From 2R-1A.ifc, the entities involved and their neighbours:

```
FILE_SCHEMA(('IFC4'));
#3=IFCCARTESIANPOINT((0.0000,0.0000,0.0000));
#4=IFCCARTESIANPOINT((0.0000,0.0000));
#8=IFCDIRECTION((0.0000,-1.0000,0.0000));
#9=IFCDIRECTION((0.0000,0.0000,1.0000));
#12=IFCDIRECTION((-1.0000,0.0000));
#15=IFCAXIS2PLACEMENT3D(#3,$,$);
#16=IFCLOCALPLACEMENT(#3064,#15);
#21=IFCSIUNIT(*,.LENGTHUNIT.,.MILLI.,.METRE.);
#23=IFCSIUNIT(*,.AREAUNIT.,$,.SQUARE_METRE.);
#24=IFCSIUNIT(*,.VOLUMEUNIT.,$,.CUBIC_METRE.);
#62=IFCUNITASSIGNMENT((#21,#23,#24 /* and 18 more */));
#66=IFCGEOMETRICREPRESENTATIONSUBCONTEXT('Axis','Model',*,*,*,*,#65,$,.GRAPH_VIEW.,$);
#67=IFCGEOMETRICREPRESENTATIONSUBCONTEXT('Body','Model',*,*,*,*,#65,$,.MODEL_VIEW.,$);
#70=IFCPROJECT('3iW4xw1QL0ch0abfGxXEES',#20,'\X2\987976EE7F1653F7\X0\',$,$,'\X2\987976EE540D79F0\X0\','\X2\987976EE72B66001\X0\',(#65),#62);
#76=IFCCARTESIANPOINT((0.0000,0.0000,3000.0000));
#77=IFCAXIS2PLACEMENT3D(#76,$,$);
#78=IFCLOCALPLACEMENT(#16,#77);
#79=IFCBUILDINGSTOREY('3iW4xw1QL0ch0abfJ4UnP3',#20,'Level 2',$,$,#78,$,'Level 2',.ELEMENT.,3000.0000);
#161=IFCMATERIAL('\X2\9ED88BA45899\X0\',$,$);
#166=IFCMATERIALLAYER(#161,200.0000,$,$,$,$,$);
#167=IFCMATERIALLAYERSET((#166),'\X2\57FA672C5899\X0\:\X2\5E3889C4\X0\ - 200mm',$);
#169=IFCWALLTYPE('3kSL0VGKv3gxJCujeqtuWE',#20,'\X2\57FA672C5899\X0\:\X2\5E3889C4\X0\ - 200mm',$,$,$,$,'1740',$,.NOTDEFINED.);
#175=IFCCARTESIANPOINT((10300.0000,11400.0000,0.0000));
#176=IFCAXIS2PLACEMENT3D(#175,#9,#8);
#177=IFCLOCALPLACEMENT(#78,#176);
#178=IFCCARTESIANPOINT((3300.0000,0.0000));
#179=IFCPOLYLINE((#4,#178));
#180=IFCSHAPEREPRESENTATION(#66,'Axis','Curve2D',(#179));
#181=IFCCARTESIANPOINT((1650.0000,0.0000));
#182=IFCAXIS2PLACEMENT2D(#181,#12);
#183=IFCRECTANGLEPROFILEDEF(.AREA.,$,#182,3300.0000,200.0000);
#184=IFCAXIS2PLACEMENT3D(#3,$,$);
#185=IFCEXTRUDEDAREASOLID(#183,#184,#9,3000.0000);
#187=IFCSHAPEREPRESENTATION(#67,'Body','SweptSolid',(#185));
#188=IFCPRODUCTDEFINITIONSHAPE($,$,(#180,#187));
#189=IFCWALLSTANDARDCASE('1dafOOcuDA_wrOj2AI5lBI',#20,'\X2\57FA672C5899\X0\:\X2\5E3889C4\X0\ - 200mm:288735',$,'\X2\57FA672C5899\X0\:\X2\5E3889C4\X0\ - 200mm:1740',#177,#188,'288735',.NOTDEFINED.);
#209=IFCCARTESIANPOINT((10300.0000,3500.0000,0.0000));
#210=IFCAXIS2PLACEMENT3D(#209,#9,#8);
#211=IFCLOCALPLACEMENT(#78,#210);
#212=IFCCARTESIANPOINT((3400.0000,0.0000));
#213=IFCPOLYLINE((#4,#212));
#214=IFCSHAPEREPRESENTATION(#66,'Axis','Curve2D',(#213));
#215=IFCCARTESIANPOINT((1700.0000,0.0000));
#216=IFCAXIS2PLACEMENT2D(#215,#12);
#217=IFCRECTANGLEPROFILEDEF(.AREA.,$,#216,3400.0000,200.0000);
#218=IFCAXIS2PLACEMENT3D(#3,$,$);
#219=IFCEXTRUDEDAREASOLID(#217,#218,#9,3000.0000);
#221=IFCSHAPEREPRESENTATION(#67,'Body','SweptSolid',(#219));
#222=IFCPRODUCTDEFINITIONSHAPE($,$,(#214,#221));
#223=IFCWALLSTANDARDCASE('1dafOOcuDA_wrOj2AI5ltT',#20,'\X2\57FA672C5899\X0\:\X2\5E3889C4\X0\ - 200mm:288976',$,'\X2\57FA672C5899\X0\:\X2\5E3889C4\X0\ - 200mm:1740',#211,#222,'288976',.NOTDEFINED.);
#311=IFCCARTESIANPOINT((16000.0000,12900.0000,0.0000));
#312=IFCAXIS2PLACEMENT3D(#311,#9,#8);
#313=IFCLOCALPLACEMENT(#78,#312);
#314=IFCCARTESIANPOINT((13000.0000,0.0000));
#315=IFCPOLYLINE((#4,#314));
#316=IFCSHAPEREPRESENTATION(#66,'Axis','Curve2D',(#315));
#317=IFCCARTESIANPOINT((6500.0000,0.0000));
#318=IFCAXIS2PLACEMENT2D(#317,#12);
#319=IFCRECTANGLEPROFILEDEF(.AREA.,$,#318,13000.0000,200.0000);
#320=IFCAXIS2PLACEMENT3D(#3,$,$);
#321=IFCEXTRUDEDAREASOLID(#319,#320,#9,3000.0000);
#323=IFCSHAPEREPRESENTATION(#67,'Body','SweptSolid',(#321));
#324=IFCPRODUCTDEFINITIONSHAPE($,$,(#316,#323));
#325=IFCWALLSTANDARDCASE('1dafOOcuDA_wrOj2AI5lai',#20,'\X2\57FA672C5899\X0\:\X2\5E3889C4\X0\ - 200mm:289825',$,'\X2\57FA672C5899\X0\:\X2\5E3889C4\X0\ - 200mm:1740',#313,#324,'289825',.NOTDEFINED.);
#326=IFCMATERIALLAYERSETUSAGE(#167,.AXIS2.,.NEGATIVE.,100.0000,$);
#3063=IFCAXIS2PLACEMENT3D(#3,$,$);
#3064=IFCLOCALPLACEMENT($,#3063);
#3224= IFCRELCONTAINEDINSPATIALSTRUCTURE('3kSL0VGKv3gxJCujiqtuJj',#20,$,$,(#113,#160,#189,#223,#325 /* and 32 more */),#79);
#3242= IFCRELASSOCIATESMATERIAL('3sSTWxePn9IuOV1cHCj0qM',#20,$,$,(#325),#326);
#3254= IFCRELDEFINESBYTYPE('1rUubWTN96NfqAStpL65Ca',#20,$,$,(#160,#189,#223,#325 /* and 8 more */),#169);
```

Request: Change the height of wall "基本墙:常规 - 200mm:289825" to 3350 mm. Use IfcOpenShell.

```python
import ifcopenshell
import ifcopenshell.geom
import ifcopenshell.util.representation
import ifcopenshell.util.shape
import ifcopenshell.util.unit

model = ifcopenshell.open("2R-1A.ifc")
unit_scale = ifcopenshell.util.unit.calculate_unit_scale(model)
settings = ifcopenshell.geom.settings()


def volume(element):
    """Net volume in cubic metres, openings subtracted."""
    shape = ifcopenshell.geom.create_shape(settings, element)
    return ifcopenshell.util.shape.get_volume(shape.geometry)


wall = model.by_id(325)
before = volume(wall)

body = ifcopenshell.util.representation.get_representation(wall, "Model", "Body")
solid = body.Items[0]
old_height = solid.Depth
solid.Depth = 3.35 / unit_scale
after = volume(wall)

print(f"height {old_height:g} -> {solid.Depth:g}, volume {before:.3f} -> {after:.3f} m3")

model.write("2R-1A-out.ifc")
```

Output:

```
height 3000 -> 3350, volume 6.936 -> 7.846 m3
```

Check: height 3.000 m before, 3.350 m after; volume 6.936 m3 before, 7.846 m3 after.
